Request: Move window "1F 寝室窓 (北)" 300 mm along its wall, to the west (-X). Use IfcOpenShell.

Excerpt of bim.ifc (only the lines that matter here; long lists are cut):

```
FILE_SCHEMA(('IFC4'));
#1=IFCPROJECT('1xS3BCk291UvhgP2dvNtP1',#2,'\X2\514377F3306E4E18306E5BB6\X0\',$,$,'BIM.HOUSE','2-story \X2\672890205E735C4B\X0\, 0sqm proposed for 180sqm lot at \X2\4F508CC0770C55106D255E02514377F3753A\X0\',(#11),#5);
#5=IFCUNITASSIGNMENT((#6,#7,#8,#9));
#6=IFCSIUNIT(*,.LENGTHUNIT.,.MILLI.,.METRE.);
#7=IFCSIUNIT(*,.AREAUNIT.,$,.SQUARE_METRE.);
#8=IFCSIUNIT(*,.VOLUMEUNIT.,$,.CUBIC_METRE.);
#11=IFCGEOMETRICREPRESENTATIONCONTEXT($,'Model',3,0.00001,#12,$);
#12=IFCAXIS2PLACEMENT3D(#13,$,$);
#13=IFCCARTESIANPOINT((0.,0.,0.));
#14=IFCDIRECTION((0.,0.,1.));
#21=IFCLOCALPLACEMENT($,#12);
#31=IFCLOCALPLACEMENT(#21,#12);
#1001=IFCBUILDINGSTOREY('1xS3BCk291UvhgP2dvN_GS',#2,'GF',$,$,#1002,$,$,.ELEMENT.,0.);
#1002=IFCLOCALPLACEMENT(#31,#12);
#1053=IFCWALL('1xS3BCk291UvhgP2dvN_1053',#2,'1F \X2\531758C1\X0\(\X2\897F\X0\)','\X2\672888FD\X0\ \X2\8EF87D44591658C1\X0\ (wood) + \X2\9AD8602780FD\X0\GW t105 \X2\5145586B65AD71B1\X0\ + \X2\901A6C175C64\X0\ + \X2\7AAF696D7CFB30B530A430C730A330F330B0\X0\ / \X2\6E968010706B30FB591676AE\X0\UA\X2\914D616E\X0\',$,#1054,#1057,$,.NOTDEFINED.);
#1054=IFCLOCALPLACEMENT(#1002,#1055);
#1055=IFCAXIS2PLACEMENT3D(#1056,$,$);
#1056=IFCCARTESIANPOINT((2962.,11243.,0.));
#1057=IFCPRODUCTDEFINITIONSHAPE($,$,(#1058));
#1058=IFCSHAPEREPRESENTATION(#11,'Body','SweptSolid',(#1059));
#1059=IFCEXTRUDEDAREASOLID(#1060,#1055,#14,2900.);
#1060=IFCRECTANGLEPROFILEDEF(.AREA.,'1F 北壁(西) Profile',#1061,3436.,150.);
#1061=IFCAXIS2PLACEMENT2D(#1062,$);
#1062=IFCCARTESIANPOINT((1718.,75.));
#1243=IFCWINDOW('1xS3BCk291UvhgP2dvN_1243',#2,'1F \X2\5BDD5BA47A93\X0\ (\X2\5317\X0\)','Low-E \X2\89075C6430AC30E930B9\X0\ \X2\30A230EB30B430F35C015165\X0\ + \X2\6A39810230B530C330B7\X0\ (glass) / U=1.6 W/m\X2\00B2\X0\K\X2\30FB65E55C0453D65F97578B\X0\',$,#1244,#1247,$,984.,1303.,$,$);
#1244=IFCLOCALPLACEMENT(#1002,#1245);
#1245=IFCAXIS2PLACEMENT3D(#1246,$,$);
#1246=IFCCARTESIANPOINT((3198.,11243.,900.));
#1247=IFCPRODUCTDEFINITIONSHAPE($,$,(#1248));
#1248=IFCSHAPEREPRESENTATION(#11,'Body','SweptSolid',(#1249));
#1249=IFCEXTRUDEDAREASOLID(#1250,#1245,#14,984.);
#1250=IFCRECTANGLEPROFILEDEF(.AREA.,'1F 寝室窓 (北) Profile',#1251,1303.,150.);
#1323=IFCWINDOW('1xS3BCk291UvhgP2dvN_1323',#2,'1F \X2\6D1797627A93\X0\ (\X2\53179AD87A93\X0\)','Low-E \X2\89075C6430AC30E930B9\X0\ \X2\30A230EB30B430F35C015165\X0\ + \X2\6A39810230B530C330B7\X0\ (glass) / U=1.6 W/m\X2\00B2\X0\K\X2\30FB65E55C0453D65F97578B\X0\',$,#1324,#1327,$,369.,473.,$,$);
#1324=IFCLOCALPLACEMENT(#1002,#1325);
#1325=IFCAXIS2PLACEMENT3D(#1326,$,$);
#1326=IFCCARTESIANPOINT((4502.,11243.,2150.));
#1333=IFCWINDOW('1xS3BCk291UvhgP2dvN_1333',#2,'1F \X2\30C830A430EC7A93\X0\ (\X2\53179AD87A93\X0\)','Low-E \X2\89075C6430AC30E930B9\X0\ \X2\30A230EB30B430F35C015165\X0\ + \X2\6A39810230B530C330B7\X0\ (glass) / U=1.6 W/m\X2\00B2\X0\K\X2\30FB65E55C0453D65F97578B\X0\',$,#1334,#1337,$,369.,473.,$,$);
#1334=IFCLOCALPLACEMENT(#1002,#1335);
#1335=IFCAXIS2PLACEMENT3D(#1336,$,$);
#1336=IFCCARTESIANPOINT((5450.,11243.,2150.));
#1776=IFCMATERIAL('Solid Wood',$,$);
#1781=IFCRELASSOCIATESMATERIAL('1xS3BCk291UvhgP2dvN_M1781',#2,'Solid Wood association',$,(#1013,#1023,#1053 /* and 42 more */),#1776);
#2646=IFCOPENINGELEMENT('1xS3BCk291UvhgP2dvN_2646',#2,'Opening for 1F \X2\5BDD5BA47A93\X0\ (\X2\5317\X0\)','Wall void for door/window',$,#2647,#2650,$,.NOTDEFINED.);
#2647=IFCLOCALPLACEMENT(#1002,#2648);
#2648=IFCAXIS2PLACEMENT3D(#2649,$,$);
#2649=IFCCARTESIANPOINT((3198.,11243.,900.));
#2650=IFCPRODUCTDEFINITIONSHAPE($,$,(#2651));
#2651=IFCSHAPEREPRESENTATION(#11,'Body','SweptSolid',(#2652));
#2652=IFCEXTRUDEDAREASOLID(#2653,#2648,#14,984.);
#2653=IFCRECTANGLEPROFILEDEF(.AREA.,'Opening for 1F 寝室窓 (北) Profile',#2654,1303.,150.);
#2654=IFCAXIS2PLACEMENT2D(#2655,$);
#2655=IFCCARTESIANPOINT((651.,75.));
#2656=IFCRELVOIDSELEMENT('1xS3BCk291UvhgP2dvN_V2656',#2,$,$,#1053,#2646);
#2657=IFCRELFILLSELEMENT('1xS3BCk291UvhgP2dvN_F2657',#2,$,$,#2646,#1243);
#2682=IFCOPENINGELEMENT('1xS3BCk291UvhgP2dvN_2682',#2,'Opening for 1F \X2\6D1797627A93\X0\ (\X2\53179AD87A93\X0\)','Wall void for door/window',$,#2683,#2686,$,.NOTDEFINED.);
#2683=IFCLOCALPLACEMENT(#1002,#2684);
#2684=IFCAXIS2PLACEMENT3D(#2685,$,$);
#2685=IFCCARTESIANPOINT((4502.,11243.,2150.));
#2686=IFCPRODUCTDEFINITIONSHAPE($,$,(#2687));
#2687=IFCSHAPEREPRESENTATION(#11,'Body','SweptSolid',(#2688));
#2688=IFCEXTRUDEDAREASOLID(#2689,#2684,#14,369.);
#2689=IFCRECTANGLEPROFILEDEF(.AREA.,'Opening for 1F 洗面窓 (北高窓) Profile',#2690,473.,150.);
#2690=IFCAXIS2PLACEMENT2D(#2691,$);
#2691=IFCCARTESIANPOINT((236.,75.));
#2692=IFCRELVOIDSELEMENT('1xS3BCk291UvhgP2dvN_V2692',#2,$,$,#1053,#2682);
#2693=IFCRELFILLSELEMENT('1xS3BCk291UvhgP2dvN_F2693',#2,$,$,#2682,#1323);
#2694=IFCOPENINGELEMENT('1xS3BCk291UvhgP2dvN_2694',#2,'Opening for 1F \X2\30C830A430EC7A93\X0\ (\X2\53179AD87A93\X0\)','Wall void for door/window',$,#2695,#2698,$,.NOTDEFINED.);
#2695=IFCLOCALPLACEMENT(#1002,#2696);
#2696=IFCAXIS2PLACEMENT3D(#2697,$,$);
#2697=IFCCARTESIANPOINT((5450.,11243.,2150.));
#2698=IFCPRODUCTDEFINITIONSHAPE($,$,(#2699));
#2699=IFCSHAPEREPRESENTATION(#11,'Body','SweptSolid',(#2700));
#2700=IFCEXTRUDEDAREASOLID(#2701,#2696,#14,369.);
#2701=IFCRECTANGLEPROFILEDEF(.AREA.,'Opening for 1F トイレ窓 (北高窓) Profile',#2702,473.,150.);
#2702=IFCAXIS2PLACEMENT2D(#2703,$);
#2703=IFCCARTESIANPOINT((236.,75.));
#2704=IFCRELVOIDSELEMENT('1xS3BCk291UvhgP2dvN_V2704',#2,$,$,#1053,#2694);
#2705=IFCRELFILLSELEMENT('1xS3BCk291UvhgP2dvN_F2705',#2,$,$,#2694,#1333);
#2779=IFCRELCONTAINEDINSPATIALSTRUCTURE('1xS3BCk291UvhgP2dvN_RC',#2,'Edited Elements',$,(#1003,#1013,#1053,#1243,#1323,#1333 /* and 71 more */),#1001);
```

```python
import ifcopenshell
import ifcopenshell.api.geometry
import ifcopenshell.util.placement
import ifcopenshell.util.unit

model = ifcopenshell.open("bim.ifc")
unit_scale = ifcopenshell.util.unit.calculate_unit_scale(model)

window = model.by_guid("1xS3BCk291UvhgP2dvN_1243")
opening = window.FillsVoids[0].RelatingOpeningElement
wall = opening.VoidsElements[0].RelatingBuildingElement

wall_matrix = ifcopenshell.util.placement.get_local_placement(wall.ObjectPlacement)
shift = wall_matrix[:3, 0] * -0.3 / unit_scale
before = ifcopenshell.util.placement.get_local_placement(window.ObjectPlacement)[:3, 3].copy()

# The window is not placed relative to its opening, so move both.
for product in (opening, window):
    matrix = ifcopenshell.util.placement.get_local_placement(product.ObjectPlacement)
    matrix[:3, 3] += shift
    ifcopenshell.api.geometry.edit_object_placement(model, product=product, matrix=matrix, is_si=False)

after = ifcopenshell.util.placement.get_local_placement(window.ObjectPlacement)[:3, 3]
print("window moved by", (after - before).round(3) + 0.0)

model.write("bim_updated.ifc")
```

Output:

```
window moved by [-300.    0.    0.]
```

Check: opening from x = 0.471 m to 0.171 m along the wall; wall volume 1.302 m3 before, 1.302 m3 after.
